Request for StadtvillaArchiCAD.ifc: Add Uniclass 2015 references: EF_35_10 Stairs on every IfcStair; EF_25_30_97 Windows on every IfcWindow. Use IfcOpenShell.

First a look at what the model holds.

```python
import ifcopenshell

model = ifcopenshell.open("StadtvillaArchiCAD.ifc")
print(model.schema)
print("classifications:", [c.Name for c in model.by_type("IfcClassification")])
for ifc_class in ("IfcDoor", "IfcRoof", "IfcStair", "IfcWall", "IfcWindow"):
    print(ifc_class, len(model.by_type(ifc_class)))
```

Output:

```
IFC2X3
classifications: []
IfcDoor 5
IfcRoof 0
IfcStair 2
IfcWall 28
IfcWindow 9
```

```python
import ifcopenshell
import ifcopenshell.api.classification

model = ifcopenshell.open("StadtvillaArchiCAD.ifc")

# IFC2X3 requires Source and Edition and has no link from the project to the system.
system = model.create_entity("IfcClassification", Source="NBS", Edition="2015", Name="Uniclass 2015")

codes = {
    "IfcStair": ("EF_35_10", "Stairs"),
    "IfcWindow": ("EF_25_30_97", "Windows"),
}
for ifc_class, (code, name) in codes.items():
    products = model.by_type(ifc_class)
    ifcopenshell.api.classification.add_reference(
        model, products=products, classification=system, identification=code, name=name
    )
    print(code, len(products))

model.write("StadtvillaArchiCAD_edited.ifc")
```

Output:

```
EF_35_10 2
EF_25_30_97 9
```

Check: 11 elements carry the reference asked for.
